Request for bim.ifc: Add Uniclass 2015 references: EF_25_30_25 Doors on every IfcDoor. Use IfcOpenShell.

First a look at what the model holds.

```python
import ifcopenshell

model = ifcopenshell.open("bim.ifc")
print(model.schema)
print("classifications:", [c.Name for c in model.by_type("IfcClassification")])
for ifc_class in ("IfcDoor", "IfcRoof", "IfcStair", "IfcWall", "IfcWindow"):
    print(ifc_class, len(model.by_type(ifc_class)))
```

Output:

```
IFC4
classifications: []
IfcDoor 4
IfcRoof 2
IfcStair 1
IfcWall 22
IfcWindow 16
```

```python
import ifcopenshell
import ifcopenshell.api.classification

model = ifcopenshell.open("bim.ifc")

system = ifcopenshell.api.classification.add_classification(model, classification="Uniclass 2015")

codes = {
    "IfcDoor": ("EF_25_30_25", "Doors"),
}
for ifc_class, (code, name) in codes.items():
    products = model.by_type(ifc_class)
    ifcopenshell.api.classification.add_reference(
        model, products=products, classification=system, identification=code, name=name
    )
    print(code, len(products))

model.write("bim_edited.ifc")
```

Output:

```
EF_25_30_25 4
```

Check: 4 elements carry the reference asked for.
